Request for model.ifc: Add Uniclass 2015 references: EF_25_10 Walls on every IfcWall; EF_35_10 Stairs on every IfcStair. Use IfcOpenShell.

First a look at what the model holds.

```python
import ifcopenshell

model = ifcopenshell.open("model.ifc")
print(model.schema)
print("classifications:", [c.Name for c in model.by_type("IfcClassification")])
for ifc_class in ("IfcDoor", "IfcRoof", "IfcStair", "IfcWall", "IfcWindow"):
    print(ifc_class, len(model.by_type(ifc_class)))
```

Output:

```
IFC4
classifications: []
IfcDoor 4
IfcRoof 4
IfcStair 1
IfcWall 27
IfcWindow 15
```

```python
import ifcopenshell
import ifcopenshell.api.classification

model = ifcopenshell.open("model.ifc")

system = ifcopenshell.api.classification.add_classification(model, classification="Uniclass 2015")

codes = {
    "IfcWall": ("EF_25_10", "Walls"),
    "IfcStair": ("EF_35_10", "Stairs"),
}
for ifc_class, (code, name) in codes.items():
    products = model.by_type(ifc_class)
    ifcopenshell.api.classification.add_reference(
        model, products=products, classification=system, identification=code, name=name
    )
    print(code, len(products))

model.write("model_v2.ifc")
```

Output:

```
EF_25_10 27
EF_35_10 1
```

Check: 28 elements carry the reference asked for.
